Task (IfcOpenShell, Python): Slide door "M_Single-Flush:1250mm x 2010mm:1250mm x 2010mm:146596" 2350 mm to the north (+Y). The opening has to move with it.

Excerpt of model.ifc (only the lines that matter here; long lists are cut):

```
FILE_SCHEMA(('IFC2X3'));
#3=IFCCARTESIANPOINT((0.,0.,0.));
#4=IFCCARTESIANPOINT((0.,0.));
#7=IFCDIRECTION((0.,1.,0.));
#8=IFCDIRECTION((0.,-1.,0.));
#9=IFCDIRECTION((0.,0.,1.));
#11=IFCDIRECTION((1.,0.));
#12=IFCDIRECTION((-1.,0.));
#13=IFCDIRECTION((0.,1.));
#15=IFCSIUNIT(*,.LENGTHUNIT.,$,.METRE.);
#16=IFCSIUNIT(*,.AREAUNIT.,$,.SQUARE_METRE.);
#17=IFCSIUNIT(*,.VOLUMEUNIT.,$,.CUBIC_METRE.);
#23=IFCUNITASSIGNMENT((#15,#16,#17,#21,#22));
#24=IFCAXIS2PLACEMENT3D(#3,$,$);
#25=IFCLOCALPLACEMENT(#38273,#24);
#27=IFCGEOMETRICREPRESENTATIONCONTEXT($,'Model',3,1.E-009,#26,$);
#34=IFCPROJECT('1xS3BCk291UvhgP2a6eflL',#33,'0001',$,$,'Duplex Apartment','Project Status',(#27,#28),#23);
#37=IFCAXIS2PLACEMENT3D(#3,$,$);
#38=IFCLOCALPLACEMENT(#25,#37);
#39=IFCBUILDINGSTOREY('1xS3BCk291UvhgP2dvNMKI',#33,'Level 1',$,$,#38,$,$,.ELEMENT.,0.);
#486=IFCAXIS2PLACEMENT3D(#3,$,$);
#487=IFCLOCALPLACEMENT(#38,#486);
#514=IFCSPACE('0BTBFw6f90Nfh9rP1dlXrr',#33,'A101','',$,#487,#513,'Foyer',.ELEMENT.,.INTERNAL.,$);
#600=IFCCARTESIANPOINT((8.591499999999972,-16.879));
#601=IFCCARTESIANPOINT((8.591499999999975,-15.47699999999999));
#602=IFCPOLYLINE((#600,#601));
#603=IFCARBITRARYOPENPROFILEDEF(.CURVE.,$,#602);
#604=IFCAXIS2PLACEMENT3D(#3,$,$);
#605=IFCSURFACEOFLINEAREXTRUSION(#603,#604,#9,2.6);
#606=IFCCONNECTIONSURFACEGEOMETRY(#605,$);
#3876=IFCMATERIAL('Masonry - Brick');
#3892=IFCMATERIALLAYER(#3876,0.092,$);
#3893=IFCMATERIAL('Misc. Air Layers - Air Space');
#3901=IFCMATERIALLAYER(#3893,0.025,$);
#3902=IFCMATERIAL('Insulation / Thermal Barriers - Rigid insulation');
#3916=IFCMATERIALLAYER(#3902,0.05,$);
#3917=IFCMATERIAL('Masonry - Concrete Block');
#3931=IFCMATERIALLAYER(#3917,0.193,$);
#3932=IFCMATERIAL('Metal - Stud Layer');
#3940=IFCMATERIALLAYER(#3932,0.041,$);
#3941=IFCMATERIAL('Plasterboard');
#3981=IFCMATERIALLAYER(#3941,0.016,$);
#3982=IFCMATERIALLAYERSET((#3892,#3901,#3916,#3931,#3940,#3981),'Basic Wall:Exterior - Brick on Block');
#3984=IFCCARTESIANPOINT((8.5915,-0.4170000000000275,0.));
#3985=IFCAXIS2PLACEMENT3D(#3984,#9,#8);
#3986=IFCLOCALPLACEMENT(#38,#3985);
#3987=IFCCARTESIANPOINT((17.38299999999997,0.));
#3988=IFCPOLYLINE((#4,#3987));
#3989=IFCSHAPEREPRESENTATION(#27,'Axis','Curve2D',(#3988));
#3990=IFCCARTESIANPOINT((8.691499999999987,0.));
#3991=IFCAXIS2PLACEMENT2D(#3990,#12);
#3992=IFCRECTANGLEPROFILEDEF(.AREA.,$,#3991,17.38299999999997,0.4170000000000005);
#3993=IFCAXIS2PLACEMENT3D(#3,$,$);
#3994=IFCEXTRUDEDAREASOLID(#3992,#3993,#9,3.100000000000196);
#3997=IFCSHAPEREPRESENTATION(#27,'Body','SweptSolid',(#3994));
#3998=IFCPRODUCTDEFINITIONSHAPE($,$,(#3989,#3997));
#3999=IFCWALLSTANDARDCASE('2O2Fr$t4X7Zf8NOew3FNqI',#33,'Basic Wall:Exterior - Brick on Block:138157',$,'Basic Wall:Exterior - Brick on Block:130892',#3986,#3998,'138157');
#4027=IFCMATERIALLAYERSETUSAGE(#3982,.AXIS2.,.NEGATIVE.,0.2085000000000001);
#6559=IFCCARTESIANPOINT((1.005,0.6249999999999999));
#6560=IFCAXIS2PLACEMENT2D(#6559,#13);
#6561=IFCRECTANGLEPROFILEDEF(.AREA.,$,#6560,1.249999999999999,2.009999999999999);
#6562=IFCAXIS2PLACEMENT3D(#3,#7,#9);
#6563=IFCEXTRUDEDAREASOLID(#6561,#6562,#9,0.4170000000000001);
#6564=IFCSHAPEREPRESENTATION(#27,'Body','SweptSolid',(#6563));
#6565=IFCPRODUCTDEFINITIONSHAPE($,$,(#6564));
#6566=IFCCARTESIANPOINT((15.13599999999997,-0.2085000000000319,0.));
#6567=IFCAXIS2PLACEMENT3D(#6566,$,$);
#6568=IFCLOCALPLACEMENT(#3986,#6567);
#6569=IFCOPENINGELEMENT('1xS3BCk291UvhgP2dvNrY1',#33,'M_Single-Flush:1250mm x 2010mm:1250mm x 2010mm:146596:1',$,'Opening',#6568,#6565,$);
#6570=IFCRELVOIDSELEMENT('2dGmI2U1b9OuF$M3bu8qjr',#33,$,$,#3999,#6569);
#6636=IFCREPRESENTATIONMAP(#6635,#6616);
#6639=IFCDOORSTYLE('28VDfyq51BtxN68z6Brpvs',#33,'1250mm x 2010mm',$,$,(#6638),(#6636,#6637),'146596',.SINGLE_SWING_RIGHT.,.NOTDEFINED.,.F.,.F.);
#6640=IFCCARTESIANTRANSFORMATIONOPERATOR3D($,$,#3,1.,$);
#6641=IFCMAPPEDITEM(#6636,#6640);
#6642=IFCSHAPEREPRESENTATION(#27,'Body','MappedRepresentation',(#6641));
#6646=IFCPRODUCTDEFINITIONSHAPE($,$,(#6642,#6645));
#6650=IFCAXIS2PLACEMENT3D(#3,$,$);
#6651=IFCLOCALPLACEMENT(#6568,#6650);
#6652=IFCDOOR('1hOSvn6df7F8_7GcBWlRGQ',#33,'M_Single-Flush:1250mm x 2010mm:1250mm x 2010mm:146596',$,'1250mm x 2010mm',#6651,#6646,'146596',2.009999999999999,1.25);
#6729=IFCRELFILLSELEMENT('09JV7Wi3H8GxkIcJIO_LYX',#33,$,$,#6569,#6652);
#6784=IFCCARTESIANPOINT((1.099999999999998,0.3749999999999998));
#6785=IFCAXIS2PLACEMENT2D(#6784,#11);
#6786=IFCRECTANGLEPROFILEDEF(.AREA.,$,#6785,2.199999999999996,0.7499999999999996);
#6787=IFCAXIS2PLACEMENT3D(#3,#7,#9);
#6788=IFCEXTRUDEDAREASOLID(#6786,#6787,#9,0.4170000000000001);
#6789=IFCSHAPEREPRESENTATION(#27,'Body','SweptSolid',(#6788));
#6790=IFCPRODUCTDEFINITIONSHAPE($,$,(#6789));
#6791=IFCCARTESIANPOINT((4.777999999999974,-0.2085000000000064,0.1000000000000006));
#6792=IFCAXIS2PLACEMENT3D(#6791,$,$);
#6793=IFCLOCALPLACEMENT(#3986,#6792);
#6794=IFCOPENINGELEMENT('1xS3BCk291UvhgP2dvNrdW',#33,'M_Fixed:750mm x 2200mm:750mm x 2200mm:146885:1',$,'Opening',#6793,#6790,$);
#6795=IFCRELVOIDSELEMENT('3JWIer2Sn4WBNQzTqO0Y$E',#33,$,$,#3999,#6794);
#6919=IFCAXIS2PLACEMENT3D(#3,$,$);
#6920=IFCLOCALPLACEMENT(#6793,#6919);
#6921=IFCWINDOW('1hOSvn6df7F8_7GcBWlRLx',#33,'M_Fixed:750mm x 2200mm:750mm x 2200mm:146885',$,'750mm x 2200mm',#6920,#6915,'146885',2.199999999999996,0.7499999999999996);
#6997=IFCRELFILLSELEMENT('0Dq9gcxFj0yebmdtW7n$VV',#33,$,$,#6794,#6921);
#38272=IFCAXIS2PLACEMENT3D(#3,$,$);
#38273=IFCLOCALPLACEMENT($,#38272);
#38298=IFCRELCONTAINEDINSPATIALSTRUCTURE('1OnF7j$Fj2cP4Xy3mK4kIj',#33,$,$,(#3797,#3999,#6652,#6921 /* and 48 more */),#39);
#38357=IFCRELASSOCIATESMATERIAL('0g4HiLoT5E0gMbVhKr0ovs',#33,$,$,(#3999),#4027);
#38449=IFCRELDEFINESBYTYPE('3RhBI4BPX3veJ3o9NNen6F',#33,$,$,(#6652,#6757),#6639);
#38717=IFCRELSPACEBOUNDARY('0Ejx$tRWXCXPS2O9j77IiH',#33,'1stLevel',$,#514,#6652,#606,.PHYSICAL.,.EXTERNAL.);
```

```python
import numpy as np
import ifcopenshell
import ifcopenshell.api.geometry
import ifcopenshell.util.placement

model = ifcopenshell.open("model.ifc")

door = model.by_guid("1hOSvn6df7F8_7GcBWlRGQ")
opening = door.FillsVoids[0].RelatingOpeningElement
wall = opening.VoidsElements[0].RelatingBuildingElement

wall_matrix = ifcopenshell.util.placement.get_local_placement(wall.ObjectPlacement)
shift = wall_matrix[:3, 0] * -2.35
before = ifcopenshell.util.placement.get_local_placement(door.ObjectPlacement)[:3, 3].copy()

# The door is placed relative to its opening, so it follows when the opening moves.
matrix = ifcopenshell.util.placement.get_local_placement(opening.ObjectPlacement)
matrix[:3, 3] += shift
ifcopenshell.api.geometry.edit_object_placement(
    model, product=opening, matrix=matrix, is_si=False, should_transform_children=True
)

# Space boundary surfaces are stored in each space's coordinates; move them too.
for rel in door.ProvidesBoundaries:
    if not rel.ConnectionGeometry:
        continue
    surface = rel.ConnectionGeometry.SurfaceOnRelatingElement
    space_matrix = ifcopenshell.util.placement.get_local_placement(rel.RelatingSpace.ObjectPlacement)
    point = np.array(surface.Position.Location.Coordinates) + space_matrix[:3, :3].T @ shift
    surface.Position = model.createIfcAxis2Placement3D(
        model.createIfcCartesianPoint(point.tolist()), surface.Position.Axis, surface.Position.RefDirection
    )

after = ifcopenshell.util.placement.get_local_placement(door.ObjectPlacement)[:3, 3]
print("door moved by", (after - before).round(3) + 0.0)

model.write("model_rev.ifc")
```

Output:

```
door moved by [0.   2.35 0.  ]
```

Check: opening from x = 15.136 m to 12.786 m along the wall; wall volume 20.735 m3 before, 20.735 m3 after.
